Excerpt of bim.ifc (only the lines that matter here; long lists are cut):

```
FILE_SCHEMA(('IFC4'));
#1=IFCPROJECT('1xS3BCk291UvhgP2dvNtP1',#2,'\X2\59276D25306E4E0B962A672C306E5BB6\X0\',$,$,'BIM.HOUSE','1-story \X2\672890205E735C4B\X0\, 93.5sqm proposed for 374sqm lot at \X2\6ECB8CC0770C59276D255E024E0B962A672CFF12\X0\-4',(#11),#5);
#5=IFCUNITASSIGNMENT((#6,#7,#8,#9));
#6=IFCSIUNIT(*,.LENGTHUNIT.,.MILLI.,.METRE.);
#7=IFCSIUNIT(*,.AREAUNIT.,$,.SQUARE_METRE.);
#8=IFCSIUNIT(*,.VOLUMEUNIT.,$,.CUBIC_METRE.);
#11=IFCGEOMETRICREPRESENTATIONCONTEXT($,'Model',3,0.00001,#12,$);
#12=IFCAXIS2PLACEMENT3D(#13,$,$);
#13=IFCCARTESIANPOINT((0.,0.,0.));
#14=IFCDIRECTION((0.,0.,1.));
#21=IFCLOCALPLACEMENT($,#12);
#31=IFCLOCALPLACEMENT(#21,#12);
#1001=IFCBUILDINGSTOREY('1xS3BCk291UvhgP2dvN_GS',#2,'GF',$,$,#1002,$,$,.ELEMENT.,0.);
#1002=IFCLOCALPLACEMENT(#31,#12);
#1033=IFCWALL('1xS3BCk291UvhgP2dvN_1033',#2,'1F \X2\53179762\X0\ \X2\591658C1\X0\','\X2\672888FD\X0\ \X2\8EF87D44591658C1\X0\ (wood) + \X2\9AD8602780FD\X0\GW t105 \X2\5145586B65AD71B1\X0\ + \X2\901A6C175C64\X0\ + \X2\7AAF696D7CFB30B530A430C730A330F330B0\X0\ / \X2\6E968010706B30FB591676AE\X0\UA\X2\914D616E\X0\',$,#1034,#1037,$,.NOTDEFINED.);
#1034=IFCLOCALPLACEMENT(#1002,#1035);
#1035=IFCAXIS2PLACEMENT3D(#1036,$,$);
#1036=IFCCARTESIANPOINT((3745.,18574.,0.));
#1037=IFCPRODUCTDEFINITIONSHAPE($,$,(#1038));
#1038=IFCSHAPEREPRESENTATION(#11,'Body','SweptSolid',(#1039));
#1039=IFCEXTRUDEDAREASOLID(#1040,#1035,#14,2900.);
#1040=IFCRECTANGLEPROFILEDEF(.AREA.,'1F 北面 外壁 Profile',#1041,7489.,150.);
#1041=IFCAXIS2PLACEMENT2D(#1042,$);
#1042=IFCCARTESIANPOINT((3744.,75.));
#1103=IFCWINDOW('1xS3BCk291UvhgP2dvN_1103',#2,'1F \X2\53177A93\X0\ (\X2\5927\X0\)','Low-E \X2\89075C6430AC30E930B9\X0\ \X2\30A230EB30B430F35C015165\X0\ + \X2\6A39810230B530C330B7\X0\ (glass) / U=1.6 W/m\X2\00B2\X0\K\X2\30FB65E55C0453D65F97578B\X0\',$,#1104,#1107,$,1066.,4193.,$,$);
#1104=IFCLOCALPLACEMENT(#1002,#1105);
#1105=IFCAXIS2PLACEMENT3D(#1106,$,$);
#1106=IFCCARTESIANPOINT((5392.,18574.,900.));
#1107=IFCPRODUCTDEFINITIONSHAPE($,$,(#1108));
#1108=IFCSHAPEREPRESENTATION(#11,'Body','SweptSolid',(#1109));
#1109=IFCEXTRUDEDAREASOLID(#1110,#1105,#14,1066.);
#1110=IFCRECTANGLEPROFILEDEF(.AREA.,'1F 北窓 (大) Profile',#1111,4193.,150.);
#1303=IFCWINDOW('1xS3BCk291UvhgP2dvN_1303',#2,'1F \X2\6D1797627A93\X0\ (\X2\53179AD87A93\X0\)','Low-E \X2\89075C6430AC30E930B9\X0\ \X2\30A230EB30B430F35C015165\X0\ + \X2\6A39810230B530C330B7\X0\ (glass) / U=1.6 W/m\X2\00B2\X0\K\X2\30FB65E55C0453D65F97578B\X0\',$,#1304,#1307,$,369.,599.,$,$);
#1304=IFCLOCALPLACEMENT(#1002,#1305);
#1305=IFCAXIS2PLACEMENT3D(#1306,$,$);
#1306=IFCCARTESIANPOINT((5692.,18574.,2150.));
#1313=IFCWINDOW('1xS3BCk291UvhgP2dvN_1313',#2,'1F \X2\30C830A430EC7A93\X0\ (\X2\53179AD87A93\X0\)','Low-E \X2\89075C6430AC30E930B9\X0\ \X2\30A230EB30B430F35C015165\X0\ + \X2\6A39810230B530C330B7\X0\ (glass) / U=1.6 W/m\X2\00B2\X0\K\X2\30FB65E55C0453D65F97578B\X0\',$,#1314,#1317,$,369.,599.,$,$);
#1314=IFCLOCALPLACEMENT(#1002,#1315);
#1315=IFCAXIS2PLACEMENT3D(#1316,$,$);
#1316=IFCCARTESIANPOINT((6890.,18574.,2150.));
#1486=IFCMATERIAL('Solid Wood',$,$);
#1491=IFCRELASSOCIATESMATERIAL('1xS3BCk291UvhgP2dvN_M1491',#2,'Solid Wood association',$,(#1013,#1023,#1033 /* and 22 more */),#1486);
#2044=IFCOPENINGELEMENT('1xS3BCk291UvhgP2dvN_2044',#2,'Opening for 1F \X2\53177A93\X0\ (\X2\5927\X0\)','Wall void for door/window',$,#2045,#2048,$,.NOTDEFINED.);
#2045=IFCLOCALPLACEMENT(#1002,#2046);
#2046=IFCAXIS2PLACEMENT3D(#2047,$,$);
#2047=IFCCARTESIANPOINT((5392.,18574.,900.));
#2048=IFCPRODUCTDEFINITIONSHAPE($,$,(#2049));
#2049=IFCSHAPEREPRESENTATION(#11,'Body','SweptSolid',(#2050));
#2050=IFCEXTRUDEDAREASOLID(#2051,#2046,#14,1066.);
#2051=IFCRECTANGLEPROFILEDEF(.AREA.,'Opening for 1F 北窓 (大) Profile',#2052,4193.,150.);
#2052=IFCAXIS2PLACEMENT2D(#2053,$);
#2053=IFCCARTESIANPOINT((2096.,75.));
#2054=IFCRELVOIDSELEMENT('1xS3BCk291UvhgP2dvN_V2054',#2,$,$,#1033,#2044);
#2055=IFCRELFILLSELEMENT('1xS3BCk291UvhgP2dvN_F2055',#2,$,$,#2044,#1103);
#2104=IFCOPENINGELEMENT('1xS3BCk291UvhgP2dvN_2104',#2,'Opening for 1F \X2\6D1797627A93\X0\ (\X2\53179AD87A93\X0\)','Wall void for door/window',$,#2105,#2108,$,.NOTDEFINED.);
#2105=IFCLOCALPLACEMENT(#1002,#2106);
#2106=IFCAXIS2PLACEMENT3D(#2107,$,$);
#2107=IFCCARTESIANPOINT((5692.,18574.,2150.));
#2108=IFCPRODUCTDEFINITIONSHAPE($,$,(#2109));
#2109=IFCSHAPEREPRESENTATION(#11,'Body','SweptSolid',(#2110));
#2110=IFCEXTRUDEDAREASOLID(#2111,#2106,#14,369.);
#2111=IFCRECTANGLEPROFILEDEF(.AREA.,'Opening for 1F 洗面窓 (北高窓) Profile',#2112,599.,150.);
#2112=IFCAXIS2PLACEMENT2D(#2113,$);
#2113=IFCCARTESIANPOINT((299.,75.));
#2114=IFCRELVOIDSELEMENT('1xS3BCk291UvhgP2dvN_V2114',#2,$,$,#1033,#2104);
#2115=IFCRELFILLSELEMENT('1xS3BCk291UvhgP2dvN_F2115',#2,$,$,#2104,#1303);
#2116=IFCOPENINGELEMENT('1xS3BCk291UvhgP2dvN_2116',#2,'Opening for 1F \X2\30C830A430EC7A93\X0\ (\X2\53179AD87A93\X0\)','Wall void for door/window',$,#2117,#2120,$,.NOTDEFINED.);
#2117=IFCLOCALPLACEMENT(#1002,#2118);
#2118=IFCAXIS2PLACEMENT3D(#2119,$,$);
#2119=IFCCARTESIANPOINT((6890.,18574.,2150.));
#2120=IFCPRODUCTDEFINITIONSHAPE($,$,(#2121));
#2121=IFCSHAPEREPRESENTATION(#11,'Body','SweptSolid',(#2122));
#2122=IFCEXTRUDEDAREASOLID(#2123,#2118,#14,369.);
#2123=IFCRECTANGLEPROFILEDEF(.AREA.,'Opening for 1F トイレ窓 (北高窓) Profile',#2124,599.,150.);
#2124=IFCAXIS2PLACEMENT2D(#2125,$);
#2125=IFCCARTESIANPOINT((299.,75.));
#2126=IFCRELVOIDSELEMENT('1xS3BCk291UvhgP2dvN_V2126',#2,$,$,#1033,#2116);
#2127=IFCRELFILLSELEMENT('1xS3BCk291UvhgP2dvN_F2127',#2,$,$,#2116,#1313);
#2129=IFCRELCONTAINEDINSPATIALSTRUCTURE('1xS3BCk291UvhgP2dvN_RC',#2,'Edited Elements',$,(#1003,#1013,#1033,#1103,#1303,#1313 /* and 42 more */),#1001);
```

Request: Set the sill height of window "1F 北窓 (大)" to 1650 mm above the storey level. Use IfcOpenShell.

```python
import numpy as np
import ifcopenshell
import ifcopenshell.api.geometry
import ifcopenshell.geom
import ifcopenshell.util.element
import ifcopenshell.util.placement
import ifcopenshell.util.shape
import ifcopenshell.util.unit

model = ifcopenshell.open("bim.ifc")
unit_scale = ifcopenshell.util.unit.calculate_unit_scale(model)

window = model.by_guid("1xS3BCk291UvhgP2dvN_1103")
opening = window.FillsVoids[0].RelatingOpeningElement
storey = ifcopenshell.util.element.get_container(window, ifc_class="IfcBuildingStorey")
level = ifcopenshell.util.placement.get_local_placement(storey.ObjectPlacement)[2, 3]

# The opening's origin need not be at the sill, so measure its lowest point.
shape = ifcopenshell.geom.create_shape(ifcopenshell.geom.settings(), opening)
bottom = ifcopenshell.util.shape.get_shape_bottom_elevation(shape, shape.geometry) / unit_scale
dz = level + 1.65 / unit_scale - bottom

shift = np.array([0.0, 0.0, dz])
# The window is not placed relative to its opening, so move both.
for product in (opening, window):
    matrix = ifcopenshell.util.placement.get_local_placement(product.ObjectPlacement)
    matrix[:3, 3] += shift
    ifcopenshell.api.geometry.edit_object_placement(model, product=product, matrix=matrix, is_si=False)

print(f"moved by {dz * unit_scale:+.3f} m")

model.write("bim_updated.ifc")
```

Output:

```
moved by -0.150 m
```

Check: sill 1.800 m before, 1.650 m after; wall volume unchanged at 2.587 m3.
